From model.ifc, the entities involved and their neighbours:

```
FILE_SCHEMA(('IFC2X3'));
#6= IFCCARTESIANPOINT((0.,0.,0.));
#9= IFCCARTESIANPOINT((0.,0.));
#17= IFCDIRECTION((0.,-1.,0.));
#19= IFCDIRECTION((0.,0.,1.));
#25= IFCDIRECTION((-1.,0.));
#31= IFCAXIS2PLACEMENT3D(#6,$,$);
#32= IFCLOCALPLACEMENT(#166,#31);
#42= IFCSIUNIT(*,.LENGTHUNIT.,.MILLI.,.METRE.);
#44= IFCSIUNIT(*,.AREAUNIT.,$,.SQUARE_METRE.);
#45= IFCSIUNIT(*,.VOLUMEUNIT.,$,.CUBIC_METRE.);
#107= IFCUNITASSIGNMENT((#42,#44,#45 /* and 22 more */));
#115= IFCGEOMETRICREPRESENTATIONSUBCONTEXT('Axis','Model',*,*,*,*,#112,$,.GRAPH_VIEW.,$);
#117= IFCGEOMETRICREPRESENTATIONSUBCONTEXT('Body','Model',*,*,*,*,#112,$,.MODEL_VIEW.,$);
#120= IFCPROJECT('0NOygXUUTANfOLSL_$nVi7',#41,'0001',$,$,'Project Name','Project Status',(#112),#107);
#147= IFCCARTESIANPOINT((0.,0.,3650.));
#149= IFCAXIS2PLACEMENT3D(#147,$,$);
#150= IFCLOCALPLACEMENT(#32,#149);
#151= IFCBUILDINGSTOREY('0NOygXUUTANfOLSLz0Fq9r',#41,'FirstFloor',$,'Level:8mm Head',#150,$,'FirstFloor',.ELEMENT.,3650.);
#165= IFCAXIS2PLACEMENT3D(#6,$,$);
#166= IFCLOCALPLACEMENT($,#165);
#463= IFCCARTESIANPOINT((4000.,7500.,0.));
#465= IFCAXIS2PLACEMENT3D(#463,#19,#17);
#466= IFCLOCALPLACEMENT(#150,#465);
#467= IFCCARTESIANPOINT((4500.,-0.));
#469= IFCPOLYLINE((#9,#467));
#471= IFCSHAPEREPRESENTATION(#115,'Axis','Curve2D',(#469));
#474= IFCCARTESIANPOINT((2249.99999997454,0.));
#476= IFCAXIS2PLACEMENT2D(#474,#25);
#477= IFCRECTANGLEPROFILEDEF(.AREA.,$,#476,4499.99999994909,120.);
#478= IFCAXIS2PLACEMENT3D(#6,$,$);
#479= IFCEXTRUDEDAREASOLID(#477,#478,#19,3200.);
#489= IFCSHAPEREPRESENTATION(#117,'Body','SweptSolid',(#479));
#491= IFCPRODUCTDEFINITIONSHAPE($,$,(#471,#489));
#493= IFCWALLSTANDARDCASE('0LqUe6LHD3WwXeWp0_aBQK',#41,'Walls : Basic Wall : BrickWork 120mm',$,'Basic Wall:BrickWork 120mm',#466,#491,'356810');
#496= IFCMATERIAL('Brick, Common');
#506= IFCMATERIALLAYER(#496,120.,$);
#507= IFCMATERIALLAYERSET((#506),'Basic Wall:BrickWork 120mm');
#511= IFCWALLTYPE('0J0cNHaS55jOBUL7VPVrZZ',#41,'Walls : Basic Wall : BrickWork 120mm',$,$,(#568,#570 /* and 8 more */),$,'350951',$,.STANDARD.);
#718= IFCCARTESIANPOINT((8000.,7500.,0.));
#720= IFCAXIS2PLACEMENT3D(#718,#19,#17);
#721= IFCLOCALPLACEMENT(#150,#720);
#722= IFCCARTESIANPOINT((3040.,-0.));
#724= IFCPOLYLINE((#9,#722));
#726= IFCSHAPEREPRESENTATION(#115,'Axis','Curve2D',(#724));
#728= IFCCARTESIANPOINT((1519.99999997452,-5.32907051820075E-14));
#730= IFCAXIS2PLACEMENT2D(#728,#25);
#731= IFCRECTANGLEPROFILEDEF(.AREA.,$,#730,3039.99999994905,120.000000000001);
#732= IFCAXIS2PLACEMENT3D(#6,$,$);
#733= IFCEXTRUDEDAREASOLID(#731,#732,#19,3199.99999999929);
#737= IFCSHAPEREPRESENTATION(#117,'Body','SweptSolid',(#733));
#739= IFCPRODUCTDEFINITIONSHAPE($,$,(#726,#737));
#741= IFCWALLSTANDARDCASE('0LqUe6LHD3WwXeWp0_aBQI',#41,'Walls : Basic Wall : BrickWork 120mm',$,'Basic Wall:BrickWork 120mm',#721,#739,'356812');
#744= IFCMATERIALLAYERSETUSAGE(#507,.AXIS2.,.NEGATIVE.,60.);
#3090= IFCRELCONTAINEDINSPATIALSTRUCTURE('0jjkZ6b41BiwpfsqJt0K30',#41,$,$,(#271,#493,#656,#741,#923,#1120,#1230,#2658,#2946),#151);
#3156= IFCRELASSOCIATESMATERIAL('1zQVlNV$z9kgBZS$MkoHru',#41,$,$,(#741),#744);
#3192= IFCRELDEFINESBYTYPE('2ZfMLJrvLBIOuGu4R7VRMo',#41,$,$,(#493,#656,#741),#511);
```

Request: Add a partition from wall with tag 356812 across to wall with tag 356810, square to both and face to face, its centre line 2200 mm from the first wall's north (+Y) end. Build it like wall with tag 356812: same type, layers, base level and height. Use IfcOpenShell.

```python
import numpy as np
import ifcopenshell
import ifcopenshell.api.geometry
import ifcopenshell.api.material
import ifcopenshell.api.pset
import ifcopenshell.api.root
import ifcopenshell.api.spatial
import ifcopenshell.api.type
import ifcopenshell.geom
import ifcopenshell.util.element
import ifcopenshell.util.placement
import ifcopenshell.util.representation
import ifcopenshell.util.shape
import ifcopenshell.util.unit

model = ifcopenshell.open("model.ifc")
unit_scale = ifcopenshell.util.unit.calculate_unit_scale(model)
settings = ifcopenshell.geom.settings()
settings.set("use-world-coords", True)

start_wall = model.by_guid("0LqUe6LHD3WwXeWp0_aBQI")
end_wall = model.by_id(493)
like = model.by_id(741)
matrix = ifcopenshell.util.placement.get_local_placement(start_wall.ObjectPlacement)
matrix[:3, 3] *= unit_scale


def extent(element):
    """Bounding box in the first wall's axes, in metres."""
    shape = ifcopenshell.geom.create_shape(settings, element)
    points = (ifcopenshell.util.shape.get_vertices(shape.geometry) - matrix[:3, 3]) @ matrix[:3, :3]
    return points.min(axis=0), points.max(axis=0)


y_start = extent(start_wall)[0][1]
y_end = extent(end_wall)[1][1]
like_min, like_max = extent(like)
length, height = float(abs(y_end - y_start)), float(like_max[2] - like_min[2])
layer_set = ifcopenshell.util.element.get_material(like, should_skip_usage=True)
thickness = sum(layer.LayerThickness for layer in layer_set.MaterialLayers) * unit_scale

wall = ifcopenshell.api.root.create_entity(model, ifc_class="IfcWallStandardCase", name="New partition")
storey = ifcopenshell.util.element.get_container(like)
ifcopenshell.api.spatial.assign_container(model, products=[wall], relating_structure=storey)
ifcopenshell.api.type.assign_type(
    model, related_objects=[wall], relating_type=ifcopenshell.util.element.get_type(like), should_map_representations=False
)
rel = ifcopenshell.api.material.assign_material(
    model, products=[wall], type="IfcMaterialLayerSetUsage", material=layer_set
)
rel.RelatingMaterial.OffsetFromReferenceLine = -thickness / 2 / unit_scale
pset = ifcopenshell.api.pset.add_pset(model, product=wall, name="Pset_WallCommon")
ifcopenshell.api.pset.edit_pset(model, pset=pset, properties={"IsExternal": False, "LoadBearing": False})

# The axis runs down the middle of the wall.
axis = ifcopenshell.api.geometry.add_axis_representation(
    model, context=ifcopenshell.util.representation.get_context(model, "Model", "Axis"), axis=[(0.0, 0.0), (length, 0.0)]
)
body = ifcopenshell.api.geometry.add_wall_representation(
    model,
    context=ifcopenshell.util.representation.get_context(model, "Model", "Body", "MODEL_VIEW"),
    length=length,
    height=height,
    thickness=thickness,
    offset=-thickness / 2,
)
for representation in (axis, body):
    ifcopenshell.api.geometry.assign_representation(model, product=wall, representation=representation)

placement = matrix @ ifcopenshell.util.placement.rotation(-90, "Z")
placement[:, 3] = matrix @ np.array([extent(start_wall)[0][0] + 2.2, y_start, like_min[2], 1.0])
ifcopenshell.api.geometry.edit_object_placement(model, product=wall, matrix=placement)

print(f"partition {length:.3f} m long, {height:.3f} m high, {thickness:.3f} m thick")

model.write("model_updated.ifc")
```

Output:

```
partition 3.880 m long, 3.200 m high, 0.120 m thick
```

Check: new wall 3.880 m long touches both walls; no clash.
